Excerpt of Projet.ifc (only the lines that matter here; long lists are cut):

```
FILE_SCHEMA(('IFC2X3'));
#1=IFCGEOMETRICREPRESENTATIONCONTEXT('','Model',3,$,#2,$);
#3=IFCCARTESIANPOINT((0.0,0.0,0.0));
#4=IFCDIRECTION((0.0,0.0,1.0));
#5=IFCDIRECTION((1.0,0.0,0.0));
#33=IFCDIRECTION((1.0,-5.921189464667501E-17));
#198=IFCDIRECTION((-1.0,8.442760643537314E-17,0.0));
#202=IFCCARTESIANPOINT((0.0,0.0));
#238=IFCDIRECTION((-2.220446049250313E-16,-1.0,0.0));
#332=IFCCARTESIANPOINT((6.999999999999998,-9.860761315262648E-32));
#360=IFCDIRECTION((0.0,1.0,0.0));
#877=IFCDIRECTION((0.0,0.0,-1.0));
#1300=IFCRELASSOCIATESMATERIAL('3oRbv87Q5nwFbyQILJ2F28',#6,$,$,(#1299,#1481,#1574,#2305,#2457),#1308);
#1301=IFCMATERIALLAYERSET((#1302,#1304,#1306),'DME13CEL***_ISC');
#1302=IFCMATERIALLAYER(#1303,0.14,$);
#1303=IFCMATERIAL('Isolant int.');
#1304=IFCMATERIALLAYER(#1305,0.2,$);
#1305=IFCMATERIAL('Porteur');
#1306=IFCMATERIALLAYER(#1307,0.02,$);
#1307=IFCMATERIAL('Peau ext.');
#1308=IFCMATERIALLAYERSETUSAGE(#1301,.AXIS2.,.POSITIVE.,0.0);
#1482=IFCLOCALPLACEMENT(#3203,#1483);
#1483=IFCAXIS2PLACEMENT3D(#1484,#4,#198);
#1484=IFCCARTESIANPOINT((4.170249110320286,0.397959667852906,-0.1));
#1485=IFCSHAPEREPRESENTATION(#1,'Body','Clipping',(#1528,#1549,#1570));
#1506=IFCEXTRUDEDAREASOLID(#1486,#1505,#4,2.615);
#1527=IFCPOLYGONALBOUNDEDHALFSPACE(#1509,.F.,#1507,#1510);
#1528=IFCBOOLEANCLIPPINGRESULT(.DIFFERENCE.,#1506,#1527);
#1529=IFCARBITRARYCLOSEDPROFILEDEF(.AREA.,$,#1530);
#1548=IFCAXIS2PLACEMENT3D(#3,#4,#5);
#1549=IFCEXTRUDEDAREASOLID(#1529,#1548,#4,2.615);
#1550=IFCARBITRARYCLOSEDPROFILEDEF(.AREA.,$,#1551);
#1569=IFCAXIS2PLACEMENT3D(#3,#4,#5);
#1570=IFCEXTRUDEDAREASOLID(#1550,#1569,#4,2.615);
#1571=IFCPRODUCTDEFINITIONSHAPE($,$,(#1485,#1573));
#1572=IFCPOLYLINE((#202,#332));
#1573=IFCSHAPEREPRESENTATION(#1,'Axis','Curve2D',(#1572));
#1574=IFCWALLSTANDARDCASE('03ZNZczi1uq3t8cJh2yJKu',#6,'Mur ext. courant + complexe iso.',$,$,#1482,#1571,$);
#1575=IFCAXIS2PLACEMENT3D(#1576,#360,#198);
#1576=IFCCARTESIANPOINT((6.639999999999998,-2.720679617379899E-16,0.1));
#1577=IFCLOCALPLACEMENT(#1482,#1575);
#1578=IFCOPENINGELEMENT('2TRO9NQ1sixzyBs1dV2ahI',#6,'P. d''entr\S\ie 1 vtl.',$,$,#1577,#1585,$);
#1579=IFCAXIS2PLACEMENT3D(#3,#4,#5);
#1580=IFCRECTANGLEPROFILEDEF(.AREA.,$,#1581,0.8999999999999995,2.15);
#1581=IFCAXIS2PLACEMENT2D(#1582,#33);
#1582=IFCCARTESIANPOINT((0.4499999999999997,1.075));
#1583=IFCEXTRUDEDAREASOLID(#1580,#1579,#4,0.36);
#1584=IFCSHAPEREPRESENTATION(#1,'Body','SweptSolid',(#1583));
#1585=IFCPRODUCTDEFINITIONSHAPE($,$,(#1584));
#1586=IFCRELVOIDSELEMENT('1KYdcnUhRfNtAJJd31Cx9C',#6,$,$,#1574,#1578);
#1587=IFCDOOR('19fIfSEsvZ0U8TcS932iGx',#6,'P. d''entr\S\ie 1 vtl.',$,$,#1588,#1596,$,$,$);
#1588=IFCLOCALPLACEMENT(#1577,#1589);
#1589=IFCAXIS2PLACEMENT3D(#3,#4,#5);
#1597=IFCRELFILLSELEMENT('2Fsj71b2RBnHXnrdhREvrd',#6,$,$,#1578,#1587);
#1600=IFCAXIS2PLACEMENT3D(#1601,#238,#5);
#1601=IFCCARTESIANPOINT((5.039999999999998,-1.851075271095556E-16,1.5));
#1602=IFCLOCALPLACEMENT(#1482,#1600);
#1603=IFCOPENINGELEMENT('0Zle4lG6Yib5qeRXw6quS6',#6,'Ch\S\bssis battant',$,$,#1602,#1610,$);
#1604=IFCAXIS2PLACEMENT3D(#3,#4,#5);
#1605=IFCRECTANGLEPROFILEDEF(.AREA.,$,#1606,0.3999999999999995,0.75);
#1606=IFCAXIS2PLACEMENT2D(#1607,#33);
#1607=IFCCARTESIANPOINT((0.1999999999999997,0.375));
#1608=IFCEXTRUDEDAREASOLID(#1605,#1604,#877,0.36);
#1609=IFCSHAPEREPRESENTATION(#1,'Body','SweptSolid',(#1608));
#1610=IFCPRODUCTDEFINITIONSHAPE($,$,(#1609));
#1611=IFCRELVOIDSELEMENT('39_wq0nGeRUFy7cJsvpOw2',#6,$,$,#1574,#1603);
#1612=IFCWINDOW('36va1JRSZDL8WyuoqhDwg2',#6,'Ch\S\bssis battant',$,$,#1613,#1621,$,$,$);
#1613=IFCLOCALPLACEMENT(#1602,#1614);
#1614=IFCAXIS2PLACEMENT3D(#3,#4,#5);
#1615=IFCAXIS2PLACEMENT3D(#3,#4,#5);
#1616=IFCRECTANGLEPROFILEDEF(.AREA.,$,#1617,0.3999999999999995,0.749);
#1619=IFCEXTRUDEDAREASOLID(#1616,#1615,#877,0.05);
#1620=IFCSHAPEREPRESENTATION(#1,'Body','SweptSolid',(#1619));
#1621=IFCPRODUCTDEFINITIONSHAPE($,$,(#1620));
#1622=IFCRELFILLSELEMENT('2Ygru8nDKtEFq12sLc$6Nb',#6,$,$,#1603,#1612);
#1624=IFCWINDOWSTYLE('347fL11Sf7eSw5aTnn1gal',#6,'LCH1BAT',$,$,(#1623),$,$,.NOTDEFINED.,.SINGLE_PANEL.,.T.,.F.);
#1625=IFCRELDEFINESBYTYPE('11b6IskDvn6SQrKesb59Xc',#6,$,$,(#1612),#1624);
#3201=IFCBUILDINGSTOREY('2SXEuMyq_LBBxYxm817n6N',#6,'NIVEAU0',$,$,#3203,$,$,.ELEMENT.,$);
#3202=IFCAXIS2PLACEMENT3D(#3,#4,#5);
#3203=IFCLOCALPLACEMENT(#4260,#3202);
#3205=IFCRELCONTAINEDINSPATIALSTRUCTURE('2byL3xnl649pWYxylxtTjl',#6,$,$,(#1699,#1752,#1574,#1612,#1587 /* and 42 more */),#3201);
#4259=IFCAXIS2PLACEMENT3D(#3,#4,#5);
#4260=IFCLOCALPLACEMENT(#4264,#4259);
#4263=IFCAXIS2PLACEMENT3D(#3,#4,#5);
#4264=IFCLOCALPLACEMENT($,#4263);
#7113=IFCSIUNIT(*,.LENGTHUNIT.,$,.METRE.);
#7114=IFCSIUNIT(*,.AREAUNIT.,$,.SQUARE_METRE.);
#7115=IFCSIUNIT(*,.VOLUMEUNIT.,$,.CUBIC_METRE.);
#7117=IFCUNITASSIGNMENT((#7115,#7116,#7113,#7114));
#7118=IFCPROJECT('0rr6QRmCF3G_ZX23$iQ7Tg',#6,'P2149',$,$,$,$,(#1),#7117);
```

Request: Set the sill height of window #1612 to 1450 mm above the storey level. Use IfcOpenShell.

```python
import numpy as np
import ifcopenshell
import ifcopenshell.api.geometry
import ifcopenshell.geom
import ifcopenshell.util.element
import ifcopenshell.util.placement
import ifcopenshell.util.shape
import ifcopenshell.util.unit

model = ifcopenshell.open("Projet.ifc")
unit_scale = ifcopenshell.util.unit.calculate_unit_scale(model)

window = model.by_guid("36va1JRSZDL8WyuoqhDwg2")
opening = window.FillsVoids[0].RelatingOpeningElement
storey = ifcopenshell.util.element.get_container(window, ifc_class="IfcBuildingStorey")
level = ifcopenshell.util.placement.get_local_placement(storey.ObjectPlacement)[2, 3]

# The opening's origin need not be at the sill, so measure its lowest point.
shape = ifcopenshell.geom.create_shape(ifcopenshell.geom.settings(), opening)
bottom = ifcopenshell.util.shape.get_shape_bottom_elevation(shape, shape.geometry) / unit_scale
dz = level + 1.45 - bottom

shift = np.array([0.0, 0.0, dz])
# The window is placed relative to its opening, so it follows when the opening moves.
matrix = ifcopenshell.util.placement.get_local_placement(opening.ObjectPlacement)
matrix[:3, 3] += shift
ifcopenshell.api.geometry.edit_object_placement(
    model, product=opening, matrix=matrix, is_si=False, should_transform_children=True
)

print(f"moved by {dz * unit_scale:+.3f} m")

model.write("Projet_rev.ifc")
```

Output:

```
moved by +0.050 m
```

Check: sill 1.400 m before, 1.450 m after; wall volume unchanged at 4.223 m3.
